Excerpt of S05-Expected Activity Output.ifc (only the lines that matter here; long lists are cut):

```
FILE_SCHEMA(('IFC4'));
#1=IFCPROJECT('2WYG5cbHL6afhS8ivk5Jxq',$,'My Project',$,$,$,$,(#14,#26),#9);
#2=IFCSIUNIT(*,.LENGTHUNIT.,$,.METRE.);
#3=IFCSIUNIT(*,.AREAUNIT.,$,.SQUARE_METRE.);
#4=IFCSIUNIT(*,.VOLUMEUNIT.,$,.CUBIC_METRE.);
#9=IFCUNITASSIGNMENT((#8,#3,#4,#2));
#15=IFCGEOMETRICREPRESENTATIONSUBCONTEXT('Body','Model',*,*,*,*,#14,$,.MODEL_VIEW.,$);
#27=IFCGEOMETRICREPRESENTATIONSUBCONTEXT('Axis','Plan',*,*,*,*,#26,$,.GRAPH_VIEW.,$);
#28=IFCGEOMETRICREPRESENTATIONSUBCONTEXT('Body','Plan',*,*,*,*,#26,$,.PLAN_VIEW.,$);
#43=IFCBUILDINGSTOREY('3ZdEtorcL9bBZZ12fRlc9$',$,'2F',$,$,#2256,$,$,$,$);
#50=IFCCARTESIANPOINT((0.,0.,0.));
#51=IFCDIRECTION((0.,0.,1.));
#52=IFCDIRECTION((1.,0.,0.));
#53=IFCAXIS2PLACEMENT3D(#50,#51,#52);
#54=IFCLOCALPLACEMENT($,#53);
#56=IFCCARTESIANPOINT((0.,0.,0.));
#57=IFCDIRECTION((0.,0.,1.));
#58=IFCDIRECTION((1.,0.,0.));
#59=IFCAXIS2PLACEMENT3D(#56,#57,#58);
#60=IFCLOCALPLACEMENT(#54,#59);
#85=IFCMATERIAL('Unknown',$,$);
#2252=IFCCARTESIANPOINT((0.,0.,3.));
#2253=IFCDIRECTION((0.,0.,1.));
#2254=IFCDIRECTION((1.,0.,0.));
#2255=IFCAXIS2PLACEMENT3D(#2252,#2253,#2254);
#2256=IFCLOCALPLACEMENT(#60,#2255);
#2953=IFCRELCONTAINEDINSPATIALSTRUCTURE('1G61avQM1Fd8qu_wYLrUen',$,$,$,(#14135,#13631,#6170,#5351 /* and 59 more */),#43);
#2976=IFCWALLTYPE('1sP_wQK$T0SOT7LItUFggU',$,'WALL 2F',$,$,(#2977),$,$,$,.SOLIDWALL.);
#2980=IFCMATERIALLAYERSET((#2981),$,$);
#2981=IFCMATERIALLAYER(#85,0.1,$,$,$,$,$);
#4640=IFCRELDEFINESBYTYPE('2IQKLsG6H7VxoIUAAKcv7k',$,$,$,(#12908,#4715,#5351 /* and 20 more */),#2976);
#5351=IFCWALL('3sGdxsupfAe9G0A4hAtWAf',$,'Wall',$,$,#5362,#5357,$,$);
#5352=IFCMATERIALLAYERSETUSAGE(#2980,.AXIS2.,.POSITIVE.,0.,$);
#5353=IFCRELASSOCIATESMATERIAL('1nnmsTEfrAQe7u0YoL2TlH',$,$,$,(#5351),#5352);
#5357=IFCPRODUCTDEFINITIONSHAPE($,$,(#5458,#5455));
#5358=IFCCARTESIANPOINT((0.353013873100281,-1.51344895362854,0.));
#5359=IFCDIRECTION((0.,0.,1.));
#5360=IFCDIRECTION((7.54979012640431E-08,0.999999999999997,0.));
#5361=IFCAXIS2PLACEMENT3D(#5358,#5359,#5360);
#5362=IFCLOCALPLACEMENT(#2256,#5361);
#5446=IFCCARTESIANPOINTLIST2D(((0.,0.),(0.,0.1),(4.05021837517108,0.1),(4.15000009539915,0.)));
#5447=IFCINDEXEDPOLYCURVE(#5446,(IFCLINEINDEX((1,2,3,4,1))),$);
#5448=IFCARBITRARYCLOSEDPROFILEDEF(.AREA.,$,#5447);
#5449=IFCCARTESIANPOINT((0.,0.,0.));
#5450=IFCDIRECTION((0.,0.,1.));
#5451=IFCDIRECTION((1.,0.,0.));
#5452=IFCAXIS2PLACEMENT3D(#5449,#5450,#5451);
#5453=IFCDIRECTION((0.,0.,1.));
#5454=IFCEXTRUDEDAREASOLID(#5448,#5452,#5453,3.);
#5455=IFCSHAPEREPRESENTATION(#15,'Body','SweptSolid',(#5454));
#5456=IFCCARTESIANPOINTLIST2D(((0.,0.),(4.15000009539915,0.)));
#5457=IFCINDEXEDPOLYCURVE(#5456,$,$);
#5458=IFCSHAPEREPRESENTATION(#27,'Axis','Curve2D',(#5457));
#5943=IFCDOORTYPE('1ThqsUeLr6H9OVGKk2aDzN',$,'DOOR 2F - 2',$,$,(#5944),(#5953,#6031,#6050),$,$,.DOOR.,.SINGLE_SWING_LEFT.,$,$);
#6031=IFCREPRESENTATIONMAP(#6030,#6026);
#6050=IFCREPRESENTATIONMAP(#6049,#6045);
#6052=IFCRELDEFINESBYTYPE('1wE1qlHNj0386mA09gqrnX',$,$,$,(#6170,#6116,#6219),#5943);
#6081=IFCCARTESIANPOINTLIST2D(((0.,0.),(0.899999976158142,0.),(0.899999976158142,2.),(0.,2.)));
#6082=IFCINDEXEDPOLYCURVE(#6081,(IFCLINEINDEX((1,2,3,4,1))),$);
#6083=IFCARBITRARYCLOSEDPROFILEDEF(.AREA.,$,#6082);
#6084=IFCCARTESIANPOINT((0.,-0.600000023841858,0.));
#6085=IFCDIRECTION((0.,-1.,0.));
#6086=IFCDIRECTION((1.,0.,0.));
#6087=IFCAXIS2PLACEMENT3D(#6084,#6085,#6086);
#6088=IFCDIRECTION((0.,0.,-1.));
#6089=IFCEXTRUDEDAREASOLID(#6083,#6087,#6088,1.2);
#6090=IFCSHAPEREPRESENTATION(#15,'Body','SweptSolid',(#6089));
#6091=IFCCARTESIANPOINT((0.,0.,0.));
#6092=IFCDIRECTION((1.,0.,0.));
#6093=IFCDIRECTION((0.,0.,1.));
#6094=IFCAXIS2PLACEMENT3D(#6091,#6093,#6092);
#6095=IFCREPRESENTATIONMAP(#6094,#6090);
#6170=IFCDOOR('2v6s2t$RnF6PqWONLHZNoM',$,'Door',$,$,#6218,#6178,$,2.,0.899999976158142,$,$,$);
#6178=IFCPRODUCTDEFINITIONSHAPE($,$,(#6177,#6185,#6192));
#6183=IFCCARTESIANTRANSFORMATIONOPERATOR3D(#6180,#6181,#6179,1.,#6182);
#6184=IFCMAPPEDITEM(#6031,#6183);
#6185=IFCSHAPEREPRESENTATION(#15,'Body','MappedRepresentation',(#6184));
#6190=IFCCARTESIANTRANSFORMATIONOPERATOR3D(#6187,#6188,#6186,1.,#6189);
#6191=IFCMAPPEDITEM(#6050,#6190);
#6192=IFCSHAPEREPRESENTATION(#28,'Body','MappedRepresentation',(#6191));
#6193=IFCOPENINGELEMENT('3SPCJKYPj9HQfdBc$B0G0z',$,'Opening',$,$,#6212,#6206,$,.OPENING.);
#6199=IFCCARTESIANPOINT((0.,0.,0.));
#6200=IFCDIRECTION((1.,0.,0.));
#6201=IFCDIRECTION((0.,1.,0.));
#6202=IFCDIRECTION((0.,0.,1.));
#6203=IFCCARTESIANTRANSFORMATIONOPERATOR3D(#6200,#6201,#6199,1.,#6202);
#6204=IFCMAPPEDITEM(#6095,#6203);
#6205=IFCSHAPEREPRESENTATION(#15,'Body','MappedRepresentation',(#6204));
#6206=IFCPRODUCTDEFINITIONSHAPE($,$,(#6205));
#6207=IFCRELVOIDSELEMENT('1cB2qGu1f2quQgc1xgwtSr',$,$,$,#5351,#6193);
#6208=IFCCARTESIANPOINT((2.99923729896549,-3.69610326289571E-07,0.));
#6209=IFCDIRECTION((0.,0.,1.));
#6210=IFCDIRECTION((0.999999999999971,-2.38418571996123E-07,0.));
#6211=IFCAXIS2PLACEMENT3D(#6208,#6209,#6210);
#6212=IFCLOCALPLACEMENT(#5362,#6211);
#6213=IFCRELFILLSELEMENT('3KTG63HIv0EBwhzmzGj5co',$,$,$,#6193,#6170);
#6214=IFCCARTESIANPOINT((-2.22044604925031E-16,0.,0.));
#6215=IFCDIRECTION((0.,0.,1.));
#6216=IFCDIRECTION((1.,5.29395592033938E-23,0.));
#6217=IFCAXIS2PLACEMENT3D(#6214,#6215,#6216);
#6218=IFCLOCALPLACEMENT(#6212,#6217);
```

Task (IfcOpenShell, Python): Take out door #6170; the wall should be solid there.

```python
import ifcopenshell
import ifcopenshell.api.feature
import ifcopenshell.api.root
import ifcopenshell.geom
import ifcopenshell.util.shape

model = ifcopenshell.open("S05-Expected Activity Output.ifc")
settings = ifcopenshell.geom.settings()


def volume(element):
    """Net volume in cubic metres, openings subtracted."""
    shape = ifcopenshell.geom.create_shape(settings, element)
    return ifcopenshell.util.shape.get_volume(shape.geometry)


door = model.by_guid("2v6s2t$RnF6PqWONLHZNoM")
opening = door.FillsVoids[0].RelatingOpeningElement
wall = opening.VoidsElements[0].RelatingBuildingElement
before = volume(wall)

ifcopenshell.api.root.remove_product(model, product=door)
ifcopenshell.api.feature.remove_feature(model, feature=opening)

after = volume(wall)

print(f"wall volume {before:.3f} -> {after:.3f} m3")

model.write("S05-Expected Activity Output-out.ifc")
```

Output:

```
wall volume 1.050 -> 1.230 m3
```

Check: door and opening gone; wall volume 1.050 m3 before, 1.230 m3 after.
